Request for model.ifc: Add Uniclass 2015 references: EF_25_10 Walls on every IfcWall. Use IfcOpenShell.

First a look at what the model holds.

```python
import ifcopenshell

model = ifcopenshell.open("model.ifc")
print(model.schema)
print("classifications:", [c.Name for c in model.by_type("IfcClassification")])
for ifc_class in ("IfcDoor", "IfcRoof", "IfcStair", "IfcWall", "IfcWindow"):
    print(ifc_class, len(model.by_type(ifc_class)))
```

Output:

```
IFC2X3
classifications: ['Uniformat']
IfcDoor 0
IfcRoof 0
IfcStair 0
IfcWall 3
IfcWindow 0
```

```python
import ifcopenshell
import ifcopenshell.api.classification

model = ifcopenshell.open("model.ifc")

# IFC2X3 requires Source and Edition and has no link from the project to the system.
system = model.create_entity("IfcClassification", Source="NBS", Edition="2015", Name="Uniclass 2015")

codes = {
    "IfcWall": ("EF_25_10", "Walls"),
}
for ifc_class, (code, name) in codes.items():
    products = model.by_type(ifc_class)
    ifcopenshell.api.classification.add_reference(
        model, products=products, classification=system, identification=code, name=name
    )
    print(code, len(products))

model.write("model_edited.ifc")
```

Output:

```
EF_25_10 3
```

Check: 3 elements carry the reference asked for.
